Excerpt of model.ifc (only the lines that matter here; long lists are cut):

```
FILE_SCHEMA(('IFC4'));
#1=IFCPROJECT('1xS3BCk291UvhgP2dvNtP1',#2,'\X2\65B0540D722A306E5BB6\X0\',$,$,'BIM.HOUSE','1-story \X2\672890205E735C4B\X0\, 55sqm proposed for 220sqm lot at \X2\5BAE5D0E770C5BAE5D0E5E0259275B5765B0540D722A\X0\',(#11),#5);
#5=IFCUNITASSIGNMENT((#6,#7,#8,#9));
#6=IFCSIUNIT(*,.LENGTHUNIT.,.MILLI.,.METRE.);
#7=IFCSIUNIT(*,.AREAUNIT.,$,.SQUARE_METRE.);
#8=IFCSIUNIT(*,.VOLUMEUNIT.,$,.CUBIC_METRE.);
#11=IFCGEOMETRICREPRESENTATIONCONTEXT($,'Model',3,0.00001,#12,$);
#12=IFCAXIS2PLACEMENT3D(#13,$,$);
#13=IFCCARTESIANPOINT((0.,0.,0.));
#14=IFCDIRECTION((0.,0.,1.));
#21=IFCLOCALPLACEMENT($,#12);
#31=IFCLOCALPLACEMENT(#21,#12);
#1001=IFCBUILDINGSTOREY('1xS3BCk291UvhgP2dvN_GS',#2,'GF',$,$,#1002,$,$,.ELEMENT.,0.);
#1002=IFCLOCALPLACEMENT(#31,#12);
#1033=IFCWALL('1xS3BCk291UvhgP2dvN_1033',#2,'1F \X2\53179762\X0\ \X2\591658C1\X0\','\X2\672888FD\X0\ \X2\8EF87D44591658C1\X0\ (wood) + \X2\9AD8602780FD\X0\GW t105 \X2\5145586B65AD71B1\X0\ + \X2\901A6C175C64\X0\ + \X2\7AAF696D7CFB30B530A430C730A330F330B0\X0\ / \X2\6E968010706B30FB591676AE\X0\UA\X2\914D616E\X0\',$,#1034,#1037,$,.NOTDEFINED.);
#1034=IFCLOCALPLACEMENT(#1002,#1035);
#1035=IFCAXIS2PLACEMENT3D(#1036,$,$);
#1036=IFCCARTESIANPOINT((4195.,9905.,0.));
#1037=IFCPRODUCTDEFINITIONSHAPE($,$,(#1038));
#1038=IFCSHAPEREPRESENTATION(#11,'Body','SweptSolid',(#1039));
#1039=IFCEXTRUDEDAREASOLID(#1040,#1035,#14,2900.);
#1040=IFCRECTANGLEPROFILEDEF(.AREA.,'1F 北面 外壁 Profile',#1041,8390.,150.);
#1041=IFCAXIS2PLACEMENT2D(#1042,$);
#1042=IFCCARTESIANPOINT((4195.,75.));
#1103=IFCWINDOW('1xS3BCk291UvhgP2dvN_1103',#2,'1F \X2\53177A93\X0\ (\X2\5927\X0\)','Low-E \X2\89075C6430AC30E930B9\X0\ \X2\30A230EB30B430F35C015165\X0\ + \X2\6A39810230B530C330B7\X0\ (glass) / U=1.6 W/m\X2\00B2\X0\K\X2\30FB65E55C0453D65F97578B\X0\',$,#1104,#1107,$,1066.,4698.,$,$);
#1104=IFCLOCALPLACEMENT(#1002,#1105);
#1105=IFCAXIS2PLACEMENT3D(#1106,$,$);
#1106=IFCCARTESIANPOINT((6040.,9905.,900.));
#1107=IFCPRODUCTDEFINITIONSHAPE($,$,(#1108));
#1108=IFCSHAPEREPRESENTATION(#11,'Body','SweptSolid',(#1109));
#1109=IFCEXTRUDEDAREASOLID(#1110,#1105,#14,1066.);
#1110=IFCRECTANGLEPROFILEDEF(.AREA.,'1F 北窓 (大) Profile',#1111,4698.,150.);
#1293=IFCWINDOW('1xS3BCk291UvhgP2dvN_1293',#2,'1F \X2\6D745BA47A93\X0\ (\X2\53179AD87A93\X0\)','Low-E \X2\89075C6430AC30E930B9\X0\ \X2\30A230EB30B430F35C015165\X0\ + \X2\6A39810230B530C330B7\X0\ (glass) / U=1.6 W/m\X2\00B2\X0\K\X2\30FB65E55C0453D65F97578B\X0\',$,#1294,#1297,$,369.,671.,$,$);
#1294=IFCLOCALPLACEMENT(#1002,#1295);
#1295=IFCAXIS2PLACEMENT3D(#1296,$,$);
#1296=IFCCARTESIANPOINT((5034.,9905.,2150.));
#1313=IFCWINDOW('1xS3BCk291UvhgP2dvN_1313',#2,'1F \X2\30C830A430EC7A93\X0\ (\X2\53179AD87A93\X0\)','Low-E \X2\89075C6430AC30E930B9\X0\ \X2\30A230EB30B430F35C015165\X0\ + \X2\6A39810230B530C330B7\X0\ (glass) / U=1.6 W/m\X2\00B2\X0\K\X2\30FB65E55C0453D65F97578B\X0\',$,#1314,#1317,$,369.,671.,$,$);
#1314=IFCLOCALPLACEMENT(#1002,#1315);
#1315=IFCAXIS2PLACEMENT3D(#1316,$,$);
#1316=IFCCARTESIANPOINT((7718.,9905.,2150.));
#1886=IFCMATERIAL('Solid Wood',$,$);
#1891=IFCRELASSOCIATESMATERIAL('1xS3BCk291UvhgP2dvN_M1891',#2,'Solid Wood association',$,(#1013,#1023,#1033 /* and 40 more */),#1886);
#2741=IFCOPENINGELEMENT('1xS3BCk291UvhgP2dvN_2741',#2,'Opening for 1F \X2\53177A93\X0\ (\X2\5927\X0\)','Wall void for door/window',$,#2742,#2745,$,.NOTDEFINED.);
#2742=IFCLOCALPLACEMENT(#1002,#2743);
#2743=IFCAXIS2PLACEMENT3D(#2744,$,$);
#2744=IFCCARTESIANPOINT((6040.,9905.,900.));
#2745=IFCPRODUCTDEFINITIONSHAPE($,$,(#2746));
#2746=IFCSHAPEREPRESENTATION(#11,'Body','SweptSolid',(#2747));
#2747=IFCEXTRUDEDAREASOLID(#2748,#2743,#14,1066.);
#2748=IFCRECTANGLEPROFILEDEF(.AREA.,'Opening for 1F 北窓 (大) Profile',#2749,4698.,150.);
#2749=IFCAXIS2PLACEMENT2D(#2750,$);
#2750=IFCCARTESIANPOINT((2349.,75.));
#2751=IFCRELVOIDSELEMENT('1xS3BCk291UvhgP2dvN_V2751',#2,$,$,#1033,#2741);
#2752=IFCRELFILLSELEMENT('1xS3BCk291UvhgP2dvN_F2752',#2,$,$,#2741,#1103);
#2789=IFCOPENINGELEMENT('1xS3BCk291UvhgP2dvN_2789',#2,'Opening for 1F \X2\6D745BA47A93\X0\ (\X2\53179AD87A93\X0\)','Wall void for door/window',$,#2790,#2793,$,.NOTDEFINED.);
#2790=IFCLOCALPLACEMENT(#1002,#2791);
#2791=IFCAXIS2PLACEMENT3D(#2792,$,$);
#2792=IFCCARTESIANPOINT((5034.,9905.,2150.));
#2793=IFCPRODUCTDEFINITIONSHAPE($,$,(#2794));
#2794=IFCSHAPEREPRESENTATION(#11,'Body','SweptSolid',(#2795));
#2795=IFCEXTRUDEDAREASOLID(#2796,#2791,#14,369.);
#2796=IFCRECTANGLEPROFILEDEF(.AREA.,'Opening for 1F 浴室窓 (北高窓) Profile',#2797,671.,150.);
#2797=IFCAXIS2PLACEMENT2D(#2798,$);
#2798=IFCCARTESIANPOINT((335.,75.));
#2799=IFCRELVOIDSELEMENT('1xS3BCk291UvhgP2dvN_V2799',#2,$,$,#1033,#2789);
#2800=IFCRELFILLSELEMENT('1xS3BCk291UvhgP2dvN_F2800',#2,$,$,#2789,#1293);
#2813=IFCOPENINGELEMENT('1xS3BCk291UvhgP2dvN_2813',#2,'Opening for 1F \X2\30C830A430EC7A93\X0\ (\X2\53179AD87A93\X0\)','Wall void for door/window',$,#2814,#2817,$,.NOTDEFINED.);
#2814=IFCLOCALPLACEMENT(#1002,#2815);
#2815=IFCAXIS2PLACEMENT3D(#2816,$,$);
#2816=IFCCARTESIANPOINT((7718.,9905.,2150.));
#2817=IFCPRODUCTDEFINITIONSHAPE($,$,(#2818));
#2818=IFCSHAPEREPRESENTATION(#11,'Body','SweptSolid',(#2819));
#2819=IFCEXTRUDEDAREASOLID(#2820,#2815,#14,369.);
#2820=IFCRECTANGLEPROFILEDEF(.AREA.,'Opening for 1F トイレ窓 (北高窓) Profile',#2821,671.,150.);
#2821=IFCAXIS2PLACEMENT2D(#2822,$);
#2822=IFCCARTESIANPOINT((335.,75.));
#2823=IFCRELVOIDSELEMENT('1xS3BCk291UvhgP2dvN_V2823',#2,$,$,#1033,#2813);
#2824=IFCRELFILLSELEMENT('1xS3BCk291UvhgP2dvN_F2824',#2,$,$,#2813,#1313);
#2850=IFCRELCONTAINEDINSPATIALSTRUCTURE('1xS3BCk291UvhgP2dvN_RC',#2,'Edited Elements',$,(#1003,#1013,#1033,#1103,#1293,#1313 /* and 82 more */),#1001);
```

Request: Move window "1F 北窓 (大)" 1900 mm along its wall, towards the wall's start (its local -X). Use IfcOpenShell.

```python
import ifcopenshell
import ifcopenshell.api.geometry
import ifcopenshell.util.placement

model = ifcopenshell.open("model.ifc")

window = model.by_guid("1xS3BCk291UvhgP2dvN_1103")
opening = window.FillsVoids[0].RelatingOpeningElement
wall = opening.VoidsElements[0].RelatingBuildingElement

wall_matrix = ifcopenshell.util.placement.get_local_placement(wall.ObjectPlacement)
shift = wall_matrix[:3, 0] * -1900.0
before = ifcopenshell.util.placement.get_local_placement(window.ObjectPlacement)[:3, 3].copy()

# The window is not placed relative to its opening, so move both.
for product in (opening, window):
    matrix = ifcopenshell.util.placement.get_local_placement(product.ObjectPlacement)
    matrix[:3, 3] += shift
    ifcopenshell.api.geometry.edit_object_placement(model, product=product, matrix=matrix, is_si=False)

after = ifcopenshell.util.placement.get_local_placement(window.ObjectPlacement)[:3, 3]
print("window moved by", (after - before).round(3) + 0.0)

model.write("model_edited.ifc")
```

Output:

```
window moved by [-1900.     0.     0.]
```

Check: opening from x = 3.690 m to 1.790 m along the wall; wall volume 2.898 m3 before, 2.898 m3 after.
